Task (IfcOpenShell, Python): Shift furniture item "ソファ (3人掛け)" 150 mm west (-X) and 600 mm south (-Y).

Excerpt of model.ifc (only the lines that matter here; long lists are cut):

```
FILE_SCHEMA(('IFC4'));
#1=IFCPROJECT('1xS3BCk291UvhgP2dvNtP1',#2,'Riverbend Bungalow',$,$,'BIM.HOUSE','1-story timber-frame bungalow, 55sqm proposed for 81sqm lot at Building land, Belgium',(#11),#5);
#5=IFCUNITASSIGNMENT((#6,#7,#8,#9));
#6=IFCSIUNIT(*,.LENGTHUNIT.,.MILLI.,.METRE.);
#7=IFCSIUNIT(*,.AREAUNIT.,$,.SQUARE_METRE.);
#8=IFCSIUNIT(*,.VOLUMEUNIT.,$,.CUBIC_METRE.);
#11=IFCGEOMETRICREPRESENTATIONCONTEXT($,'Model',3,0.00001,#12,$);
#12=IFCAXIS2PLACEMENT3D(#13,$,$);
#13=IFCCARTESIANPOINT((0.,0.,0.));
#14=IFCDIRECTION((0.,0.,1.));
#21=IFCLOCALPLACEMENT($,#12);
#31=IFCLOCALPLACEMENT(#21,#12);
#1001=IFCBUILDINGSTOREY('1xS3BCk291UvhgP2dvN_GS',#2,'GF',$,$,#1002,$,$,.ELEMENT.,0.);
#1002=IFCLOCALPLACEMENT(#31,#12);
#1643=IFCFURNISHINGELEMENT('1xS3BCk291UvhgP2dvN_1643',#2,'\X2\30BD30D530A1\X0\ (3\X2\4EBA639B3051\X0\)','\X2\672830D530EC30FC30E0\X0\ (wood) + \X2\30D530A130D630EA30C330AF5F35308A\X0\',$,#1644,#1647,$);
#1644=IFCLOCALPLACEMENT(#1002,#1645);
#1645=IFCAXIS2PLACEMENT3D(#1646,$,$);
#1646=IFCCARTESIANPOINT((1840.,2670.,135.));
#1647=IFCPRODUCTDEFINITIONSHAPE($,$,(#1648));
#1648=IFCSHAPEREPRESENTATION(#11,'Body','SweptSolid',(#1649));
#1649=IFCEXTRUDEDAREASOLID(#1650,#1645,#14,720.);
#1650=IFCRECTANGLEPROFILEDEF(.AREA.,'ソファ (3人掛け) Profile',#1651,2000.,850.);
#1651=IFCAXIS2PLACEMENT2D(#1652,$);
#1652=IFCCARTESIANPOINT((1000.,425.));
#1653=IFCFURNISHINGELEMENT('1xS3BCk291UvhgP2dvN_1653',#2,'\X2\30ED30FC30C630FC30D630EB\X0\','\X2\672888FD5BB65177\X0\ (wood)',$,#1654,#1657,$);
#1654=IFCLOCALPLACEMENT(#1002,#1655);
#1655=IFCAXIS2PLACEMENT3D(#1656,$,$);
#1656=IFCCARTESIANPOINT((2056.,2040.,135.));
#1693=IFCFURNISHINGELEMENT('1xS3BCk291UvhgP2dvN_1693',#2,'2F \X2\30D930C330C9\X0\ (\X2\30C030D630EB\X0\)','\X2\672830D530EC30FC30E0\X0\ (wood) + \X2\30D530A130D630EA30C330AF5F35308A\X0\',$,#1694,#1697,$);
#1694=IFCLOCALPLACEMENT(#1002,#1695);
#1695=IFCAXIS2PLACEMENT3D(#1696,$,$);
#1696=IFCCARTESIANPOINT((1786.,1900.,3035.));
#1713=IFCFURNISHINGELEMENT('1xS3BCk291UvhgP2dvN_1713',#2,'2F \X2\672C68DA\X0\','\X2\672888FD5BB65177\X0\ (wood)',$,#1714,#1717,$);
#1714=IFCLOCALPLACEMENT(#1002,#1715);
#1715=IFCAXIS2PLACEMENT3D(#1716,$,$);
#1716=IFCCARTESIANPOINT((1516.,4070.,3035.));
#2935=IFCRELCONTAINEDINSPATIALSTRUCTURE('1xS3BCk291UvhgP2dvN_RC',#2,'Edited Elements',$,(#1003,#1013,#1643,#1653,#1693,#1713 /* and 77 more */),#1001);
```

```python
import ifcopenshell
import ifcopenshell.api.geometry
import ifcopenshell.util.placement

model = ifcopenshell.open("model.ifc")

item = model.by_guid("1xS3BCk291UvhgP2dvN_1643")
matrix = ifcopenshell.util.placement.get_local_placement(item.ObjectPlacement)
matrix[0, 3] -= 150.0
matrix[1, 3] -= 600.0
ifcopenshell.api.geometry.edit_object_placement(model, product=item, matrix=matrix, is_si=False)

print(ifcopenshell.util.placement.get_local_placement(item.ObjectPlacement).round(3) + 0.0)

model.write("model_rev.ifc")
```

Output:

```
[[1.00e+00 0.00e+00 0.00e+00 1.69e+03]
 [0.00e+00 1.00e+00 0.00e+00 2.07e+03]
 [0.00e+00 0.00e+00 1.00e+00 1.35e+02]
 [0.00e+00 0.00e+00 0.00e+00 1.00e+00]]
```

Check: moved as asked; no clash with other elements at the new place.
